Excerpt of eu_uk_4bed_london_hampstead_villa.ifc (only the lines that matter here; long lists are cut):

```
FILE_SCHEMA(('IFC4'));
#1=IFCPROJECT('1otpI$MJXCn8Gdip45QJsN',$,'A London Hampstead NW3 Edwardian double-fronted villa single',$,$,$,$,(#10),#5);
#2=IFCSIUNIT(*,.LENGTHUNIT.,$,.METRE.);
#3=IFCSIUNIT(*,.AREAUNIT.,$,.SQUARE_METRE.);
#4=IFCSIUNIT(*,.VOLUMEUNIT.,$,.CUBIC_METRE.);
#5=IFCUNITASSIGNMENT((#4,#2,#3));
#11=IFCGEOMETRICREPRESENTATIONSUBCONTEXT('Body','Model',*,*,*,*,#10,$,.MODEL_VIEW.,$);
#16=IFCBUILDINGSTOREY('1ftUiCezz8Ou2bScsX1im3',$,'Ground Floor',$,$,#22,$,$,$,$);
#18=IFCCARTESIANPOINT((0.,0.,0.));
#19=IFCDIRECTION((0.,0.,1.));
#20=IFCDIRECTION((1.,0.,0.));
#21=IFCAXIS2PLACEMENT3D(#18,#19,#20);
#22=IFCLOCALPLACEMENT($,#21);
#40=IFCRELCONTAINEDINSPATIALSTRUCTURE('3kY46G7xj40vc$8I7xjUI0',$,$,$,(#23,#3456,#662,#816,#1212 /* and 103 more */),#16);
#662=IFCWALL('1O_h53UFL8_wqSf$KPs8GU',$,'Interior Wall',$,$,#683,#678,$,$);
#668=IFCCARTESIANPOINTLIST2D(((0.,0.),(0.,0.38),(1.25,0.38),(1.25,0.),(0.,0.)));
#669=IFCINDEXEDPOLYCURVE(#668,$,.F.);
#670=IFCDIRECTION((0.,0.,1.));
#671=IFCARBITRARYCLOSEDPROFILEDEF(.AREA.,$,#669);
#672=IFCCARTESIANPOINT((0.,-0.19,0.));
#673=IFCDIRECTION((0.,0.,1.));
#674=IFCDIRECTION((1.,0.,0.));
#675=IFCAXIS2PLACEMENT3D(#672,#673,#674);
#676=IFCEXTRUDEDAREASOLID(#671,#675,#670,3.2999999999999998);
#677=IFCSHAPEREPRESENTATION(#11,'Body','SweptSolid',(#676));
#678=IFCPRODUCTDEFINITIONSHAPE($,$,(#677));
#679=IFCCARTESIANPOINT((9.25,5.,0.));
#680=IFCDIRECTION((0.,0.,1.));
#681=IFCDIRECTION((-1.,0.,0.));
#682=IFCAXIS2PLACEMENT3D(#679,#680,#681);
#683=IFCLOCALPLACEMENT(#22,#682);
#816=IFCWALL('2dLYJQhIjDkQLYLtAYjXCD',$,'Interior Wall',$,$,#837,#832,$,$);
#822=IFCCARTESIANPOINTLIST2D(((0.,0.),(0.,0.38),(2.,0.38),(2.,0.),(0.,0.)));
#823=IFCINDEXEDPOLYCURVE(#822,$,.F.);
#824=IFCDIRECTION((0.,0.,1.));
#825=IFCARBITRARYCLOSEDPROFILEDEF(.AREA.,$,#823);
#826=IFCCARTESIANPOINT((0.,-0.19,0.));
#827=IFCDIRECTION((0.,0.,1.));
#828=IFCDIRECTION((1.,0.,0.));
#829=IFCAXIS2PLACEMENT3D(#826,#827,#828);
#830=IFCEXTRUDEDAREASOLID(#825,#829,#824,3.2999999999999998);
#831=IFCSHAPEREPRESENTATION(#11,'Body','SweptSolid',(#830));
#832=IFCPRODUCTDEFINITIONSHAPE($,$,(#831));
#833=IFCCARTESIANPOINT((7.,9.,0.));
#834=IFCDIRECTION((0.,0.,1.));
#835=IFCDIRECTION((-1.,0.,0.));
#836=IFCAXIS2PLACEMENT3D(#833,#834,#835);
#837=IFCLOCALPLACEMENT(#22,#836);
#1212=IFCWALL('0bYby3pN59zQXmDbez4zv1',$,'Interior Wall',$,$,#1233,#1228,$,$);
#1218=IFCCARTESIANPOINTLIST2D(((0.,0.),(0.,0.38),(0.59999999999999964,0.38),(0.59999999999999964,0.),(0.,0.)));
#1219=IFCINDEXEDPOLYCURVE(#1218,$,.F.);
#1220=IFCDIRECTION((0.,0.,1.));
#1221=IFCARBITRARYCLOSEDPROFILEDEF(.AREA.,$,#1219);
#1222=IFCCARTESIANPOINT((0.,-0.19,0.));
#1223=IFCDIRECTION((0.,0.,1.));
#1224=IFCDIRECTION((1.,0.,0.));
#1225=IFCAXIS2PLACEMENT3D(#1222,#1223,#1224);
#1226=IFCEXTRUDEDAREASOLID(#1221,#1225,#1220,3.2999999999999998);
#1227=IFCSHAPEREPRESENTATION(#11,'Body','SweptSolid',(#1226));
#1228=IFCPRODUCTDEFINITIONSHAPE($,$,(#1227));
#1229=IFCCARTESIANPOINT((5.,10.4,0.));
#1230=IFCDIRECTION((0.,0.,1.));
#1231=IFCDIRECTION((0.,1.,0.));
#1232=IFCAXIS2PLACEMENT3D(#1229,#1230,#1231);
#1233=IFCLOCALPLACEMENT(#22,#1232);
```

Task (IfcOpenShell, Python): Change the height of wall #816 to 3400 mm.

```python
import ifcopenshell
import ifcopenshell.geom
import ifcopenshell.util.representation
import ifcopenshell.util.shape
import ifcopenshell.util.unit

model = ifcopenshell.open("eu_uk_4bed_london_hampstead_villa.ifc")
unit_scale = ifcopenshell.util.unit.calculate_unit_scale(model)
settings = ifcopenshell.geom.settings()


def volume(element):
    """Net volume in cubic metres, openings subtracted."""
    shape = ifcopenshell.geom.create_shape(settings, element)
    return ifcopenshell.util.shape.get_volume(shape.geometry)


wall = model.by_id(816)
before = volume(wall)

body = ifcopenshell.util.representation.get_representation(wall, "Model", "Body")
solid = body.Items[0]
old_height = solid.Depth
solid.Depth = 3.4 / unit_scale
after = volume(wall)

print(f"height {old_height:g} -> {solid.Depth:g}, volume {before:.3f} -> {after:.3f} m3")

model.write("eu_uk_4bed_london_hampstead_villa_updated.ifc")
```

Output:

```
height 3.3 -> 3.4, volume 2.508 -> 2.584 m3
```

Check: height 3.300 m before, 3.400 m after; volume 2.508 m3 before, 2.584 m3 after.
